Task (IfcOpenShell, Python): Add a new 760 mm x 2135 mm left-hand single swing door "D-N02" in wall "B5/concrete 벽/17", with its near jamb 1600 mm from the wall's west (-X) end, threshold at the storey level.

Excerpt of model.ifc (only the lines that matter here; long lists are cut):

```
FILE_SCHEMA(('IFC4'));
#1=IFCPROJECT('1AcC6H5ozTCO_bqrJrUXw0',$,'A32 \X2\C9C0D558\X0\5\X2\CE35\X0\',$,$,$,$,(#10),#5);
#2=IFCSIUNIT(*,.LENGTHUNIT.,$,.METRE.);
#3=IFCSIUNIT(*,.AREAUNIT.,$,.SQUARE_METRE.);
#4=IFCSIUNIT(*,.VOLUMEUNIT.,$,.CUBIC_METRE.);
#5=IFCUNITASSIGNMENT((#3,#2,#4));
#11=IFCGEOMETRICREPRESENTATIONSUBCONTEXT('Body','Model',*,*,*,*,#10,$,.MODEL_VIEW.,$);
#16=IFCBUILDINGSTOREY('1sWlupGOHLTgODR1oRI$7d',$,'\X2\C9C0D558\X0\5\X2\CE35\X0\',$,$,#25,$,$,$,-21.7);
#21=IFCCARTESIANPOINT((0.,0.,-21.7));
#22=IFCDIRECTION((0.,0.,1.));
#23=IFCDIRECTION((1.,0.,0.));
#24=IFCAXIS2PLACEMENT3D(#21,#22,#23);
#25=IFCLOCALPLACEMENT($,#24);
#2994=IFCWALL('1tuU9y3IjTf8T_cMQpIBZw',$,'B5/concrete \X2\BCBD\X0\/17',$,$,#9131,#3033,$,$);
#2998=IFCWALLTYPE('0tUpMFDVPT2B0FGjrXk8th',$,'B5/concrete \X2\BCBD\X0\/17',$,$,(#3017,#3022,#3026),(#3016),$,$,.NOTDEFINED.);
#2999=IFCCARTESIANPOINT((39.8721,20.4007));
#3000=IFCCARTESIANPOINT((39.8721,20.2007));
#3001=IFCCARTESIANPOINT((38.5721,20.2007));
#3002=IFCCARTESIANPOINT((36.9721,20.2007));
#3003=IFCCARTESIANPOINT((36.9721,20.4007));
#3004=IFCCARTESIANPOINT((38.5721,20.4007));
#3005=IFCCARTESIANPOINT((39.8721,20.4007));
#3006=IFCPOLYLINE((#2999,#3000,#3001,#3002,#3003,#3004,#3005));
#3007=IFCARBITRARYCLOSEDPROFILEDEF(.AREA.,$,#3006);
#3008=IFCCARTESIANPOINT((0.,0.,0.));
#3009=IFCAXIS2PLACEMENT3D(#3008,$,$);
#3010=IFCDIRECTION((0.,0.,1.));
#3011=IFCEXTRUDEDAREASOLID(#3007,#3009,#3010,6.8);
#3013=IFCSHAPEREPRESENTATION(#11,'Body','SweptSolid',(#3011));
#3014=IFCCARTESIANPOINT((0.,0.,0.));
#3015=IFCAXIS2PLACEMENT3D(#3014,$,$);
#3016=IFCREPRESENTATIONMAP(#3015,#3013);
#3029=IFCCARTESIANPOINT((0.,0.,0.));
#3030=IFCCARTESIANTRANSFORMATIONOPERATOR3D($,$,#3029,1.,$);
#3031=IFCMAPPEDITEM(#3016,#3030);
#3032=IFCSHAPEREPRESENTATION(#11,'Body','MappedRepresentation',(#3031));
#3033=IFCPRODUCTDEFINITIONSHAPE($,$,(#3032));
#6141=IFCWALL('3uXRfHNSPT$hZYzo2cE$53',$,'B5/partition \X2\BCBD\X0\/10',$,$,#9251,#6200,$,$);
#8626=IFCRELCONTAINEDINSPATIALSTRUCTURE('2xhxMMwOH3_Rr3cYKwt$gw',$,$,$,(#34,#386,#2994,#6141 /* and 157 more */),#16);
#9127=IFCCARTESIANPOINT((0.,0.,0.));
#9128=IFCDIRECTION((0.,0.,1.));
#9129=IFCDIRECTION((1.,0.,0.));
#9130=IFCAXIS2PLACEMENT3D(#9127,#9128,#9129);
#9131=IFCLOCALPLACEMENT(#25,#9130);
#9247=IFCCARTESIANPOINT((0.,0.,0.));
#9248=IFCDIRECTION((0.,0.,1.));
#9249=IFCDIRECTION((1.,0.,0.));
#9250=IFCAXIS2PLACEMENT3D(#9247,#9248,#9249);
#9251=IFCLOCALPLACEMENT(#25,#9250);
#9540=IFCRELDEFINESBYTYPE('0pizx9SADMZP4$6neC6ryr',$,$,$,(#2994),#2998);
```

```python
import numpy as np
import ifcopenshell
import ifcopenshell.api.feature
import ifcopenshell.api.geometry
import ifcopenshell.api.root
import ifcopenshell.api.spatial
import ifcopenshell.geom
import ifcopenshell.util.element
import ifcopenshell.util.placement
import ifcopenshell.util.representation
import ifcopenshell.util.shape
import ifcopenshell.util.unit

model = ifcopenshell.open("model.ifc")
unit_scale = ifcopenshell.util.unit.calculate_unit_scale(model)
settings = ifcopenshell.geom.settings()


def volume(element):
    """Net volume in cubic metres, openings subtracted."""
    shape = ifcopenshell.geom.create_shape(settings, element)
    return ifcopenshell.util.shape.get_volume(shape.geometry)


wall = model.by_guid("1tuU9y3IjTf8T_cMQpIBZw")
storey = ifcopenshell.util.element.get_container(wall, ifc_class="IfcBuildingStorey")
context = ifcopenshell.util.representation.get_context(model, "Model", "Body", "MODEL_VIEW")
before = volume(wall)

width, height, from_end, sill = 0.76, 2.135, 1.6, 0.0  # metres

# The wall runs along its own X axis, and the end named is its -X end.
wall_shape = ifcopenshell.geom.create_shape(settings, wall)
x, y, z = ifcopenshell.util.shape.get_vertices(wall_shape.geometry).T
start = x.min() + from_end
face, thickness = float(y.min()), float(y.max() - y.min())
wall_matrix = ifcopenshell.util.placement.get_local_placement(wall.ObjectPlacement)
level = ifcopenshell.util.placement.get_local_placement(storey.ObjectPlacement)[2, 3]


def in_wall(x, y):
    """Placement at x, y metres in the wall's axes, at sill height."""
    matrix = wall_matrix.copy()
    matrix[:, 3] = wall_matrix @ np.array([x / unit_scale, y / unit_scale, 0.0, 1.0])
    matrix[2, 3] = level + sill / unit_scale
    return matrix


# Opening: a box that overshoots both wall faces by 50 mm.
opening = ifcopenshell.api.root.create_entity(model, ifc_class="IfcOpeningElement", predefined_type="OPENING")
box = ifcopenshell.api.geometry.add_wall_representation(
    model, context=context, length=width, height=height, thickness=thickness + 0.1
)
ifcopenshell.api.geometry.assign_representation(model, product=opening, representation=box)
ifcopenshell.api.geometry.edit_object_placement(model, product=opening, matrix=in_wall(start, face - 0.05), is_si=False)
ifcopenshell.api.feature.add_feature(model, feature=opening, element=wall)

door = ifcopenshell.api.root.create_entity(model, ifc_class="IfcDoor", name="D-N02", predefined_type="DOOR")
door.OverallWidth, door.OverallHeight = width / unit_scale, height / unit_scale
door.OperationType = "SINGLE_SWING_LEFT"
body = ifcopenshell.api.geometry.add_door_representation(
    model,
    context=context,
    overall_width=door.OverallWidth,
    overall_height=door.OverallHeight,
    operation_type="SINGLE_SWING_LEFT",
    lining_properties={"LiningDepth": thickness / unit_scale, "ThresholdDepth": thickness / unit_scale},
)
ifcopenshell.api.geometry.assign_representation(model, product=door, representation=body)
ifcopenshell.api.spatial.assign_container(model, products=[door], relating_structure=storey)
ifcopenshell.api.feature.add_filling(model, opening=opening, element=door)

# The lining spans the wall, so the door starts at the wall face.
ifcopenshell.api.geometry.edit_object_placement(model, product=door, matrix=in_wall(start, face), is_si=False)

after = volume(wall)

print(f"wall volume {before:.3f} -> {after:.3f} m3")

model.write("model_updated.ifc")
```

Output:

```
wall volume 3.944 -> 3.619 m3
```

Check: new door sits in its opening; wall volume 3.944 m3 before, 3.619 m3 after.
